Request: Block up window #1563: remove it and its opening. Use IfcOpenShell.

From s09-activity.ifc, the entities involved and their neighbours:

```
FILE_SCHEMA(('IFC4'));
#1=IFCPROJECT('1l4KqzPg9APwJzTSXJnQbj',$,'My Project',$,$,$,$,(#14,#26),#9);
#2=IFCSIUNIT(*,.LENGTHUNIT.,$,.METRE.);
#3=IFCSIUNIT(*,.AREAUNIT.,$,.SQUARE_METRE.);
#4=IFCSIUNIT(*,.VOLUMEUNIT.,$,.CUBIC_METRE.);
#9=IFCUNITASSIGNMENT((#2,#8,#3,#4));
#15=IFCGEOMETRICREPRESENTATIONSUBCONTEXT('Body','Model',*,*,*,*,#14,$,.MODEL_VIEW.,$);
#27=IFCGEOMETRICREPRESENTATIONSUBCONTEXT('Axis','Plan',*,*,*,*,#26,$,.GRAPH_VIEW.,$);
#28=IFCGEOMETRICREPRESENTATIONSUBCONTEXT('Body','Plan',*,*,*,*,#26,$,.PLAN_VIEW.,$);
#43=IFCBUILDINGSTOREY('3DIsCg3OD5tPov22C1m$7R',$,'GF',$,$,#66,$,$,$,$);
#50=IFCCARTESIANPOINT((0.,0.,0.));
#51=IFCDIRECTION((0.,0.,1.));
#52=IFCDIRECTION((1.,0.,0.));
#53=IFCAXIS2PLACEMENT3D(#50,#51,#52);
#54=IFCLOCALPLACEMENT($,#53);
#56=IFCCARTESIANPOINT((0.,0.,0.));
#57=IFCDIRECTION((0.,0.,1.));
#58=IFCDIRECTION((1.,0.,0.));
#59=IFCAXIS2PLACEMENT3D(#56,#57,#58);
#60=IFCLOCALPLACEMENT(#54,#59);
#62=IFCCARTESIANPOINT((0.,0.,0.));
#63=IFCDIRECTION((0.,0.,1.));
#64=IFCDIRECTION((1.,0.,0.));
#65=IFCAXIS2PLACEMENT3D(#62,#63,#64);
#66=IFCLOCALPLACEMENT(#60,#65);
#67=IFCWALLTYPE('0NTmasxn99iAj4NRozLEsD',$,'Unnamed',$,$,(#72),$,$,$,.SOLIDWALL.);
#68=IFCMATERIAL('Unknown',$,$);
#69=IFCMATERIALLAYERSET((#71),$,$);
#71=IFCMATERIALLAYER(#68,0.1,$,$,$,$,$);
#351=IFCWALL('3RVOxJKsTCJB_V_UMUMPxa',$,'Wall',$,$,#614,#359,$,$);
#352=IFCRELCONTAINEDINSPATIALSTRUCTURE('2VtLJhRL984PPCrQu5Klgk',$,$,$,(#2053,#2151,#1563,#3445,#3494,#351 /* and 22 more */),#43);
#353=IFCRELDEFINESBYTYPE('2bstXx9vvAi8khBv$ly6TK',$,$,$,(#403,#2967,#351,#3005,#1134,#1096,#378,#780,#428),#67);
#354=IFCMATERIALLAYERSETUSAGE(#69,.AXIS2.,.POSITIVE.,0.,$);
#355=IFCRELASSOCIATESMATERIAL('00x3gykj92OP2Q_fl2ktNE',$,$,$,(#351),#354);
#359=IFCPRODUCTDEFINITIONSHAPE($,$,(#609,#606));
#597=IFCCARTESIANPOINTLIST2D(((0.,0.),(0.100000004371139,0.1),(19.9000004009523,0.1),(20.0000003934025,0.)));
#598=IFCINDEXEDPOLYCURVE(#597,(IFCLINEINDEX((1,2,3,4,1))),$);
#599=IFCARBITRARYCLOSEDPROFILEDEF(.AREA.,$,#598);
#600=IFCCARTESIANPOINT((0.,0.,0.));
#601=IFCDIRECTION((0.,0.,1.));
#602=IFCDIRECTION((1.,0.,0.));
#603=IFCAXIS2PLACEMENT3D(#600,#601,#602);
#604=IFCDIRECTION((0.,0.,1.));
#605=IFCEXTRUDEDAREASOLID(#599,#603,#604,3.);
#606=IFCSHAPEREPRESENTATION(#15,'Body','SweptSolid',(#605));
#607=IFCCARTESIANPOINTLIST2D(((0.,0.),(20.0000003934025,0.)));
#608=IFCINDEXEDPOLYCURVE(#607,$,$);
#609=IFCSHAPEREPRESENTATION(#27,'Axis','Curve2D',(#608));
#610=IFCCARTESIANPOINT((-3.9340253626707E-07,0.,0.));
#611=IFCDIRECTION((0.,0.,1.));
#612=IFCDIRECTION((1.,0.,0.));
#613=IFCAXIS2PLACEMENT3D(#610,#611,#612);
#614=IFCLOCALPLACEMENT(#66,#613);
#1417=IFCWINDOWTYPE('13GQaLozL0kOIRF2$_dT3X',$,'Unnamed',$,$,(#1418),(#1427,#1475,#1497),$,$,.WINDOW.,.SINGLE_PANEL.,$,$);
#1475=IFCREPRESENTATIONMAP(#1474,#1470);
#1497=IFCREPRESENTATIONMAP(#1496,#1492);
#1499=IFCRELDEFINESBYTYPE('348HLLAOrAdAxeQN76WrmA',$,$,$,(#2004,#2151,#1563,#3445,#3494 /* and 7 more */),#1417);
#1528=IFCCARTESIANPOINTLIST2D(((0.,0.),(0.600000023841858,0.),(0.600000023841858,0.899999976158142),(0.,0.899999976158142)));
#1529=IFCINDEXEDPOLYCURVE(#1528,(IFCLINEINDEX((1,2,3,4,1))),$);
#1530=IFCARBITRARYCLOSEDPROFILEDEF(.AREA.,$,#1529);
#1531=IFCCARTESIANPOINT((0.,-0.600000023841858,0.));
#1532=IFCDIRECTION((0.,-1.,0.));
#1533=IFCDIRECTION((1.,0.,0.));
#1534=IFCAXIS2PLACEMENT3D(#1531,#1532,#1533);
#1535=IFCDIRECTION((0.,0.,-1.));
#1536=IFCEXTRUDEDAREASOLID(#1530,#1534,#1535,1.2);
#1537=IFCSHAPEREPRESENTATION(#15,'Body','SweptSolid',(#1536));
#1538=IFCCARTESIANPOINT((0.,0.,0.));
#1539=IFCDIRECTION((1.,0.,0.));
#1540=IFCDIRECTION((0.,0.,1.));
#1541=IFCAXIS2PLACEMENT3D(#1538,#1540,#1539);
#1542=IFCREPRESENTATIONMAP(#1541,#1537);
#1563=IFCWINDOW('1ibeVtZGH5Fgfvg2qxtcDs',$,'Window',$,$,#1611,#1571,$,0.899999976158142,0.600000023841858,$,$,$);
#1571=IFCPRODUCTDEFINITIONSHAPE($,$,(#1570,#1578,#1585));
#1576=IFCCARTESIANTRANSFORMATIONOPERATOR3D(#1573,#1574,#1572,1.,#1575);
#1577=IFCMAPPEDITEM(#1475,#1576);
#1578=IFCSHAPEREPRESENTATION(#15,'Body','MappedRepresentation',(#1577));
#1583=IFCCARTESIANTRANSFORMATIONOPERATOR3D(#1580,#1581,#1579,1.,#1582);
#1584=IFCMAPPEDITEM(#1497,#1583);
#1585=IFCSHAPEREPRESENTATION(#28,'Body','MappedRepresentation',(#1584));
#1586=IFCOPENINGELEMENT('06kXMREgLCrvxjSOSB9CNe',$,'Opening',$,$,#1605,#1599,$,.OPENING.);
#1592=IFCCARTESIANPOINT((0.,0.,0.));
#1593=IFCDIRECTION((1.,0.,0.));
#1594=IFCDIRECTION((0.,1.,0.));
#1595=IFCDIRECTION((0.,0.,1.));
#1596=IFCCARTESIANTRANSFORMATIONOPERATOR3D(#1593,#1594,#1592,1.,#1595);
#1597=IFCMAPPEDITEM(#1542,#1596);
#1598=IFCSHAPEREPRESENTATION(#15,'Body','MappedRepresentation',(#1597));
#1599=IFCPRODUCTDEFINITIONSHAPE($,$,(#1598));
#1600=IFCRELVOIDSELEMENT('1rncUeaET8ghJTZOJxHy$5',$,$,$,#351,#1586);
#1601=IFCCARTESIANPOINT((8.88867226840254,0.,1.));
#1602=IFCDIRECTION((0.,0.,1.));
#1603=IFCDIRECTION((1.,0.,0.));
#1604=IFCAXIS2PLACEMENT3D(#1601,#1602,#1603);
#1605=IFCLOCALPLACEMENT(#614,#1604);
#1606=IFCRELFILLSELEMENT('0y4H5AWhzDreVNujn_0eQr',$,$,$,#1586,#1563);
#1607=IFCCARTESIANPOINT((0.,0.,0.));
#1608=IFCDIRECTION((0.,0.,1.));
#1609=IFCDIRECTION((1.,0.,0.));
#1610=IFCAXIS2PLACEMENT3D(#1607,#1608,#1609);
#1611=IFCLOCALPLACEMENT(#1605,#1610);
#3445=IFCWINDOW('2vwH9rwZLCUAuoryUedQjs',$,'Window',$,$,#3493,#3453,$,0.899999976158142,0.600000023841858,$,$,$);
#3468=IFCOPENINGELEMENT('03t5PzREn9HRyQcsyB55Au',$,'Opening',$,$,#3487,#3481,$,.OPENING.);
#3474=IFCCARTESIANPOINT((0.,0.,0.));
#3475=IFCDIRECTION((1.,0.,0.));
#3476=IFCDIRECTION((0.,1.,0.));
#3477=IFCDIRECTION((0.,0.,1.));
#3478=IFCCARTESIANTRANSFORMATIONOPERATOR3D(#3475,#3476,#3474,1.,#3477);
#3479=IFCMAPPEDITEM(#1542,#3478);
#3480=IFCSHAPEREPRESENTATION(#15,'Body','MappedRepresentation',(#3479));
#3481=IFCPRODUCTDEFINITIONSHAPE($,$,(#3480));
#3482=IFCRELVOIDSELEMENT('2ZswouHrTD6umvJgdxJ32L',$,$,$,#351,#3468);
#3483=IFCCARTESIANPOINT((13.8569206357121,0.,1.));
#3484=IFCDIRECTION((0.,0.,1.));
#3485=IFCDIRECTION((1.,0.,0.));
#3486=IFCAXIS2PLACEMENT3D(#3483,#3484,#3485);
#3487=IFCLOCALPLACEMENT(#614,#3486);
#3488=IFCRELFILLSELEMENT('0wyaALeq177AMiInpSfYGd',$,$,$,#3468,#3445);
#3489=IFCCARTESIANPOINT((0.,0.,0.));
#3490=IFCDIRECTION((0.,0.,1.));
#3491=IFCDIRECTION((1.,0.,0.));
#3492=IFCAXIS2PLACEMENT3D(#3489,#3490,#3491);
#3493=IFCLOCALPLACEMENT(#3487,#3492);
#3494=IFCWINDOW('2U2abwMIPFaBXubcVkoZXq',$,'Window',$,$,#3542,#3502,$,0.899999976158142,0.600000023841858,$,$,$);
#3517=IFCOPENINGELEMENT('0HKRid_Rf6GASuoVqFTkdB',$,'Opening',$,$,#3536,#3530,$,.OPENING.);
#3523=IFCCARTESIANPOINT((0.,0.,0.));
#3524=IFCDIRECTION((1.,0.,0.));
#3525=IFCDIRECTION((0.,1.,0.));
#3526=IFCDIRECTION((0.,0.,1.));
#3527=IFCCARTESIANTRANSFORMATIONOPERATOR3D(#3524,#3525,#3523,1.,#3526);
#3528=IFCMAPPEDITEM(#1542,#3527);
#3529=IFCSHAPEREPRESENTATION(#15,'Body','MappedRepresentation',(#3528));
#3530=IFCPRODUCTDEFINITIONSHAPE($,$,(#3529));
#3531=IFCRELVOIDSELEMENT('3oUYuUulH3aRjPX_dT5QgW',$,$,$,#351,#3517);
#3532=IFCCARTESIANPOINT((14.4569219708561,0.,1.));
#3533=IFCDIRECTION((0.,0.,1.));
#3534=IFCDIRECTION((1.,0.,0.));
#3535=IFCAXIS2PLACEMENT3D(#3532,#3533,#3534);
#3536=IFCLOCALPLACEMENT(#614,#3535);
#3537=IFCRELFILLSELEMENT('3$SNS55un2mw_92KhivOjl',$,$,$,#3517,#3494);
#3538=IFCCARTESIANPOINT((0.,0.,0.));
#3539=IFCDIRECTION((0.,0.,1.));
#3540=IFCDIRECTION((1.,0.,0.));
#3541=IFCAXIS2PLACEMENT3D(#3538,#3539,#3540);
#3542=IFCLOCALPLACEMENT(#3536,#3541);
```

```python
import ifcopenshell
import ifcopenshell.api.feature
import ifcopenshell.api.root
import ifcopenshell.geom
import ifcopenshell.util.shape

model = ifcopenshell.open("s09-activity.ifc")
settings = ifcopenshell.geom.settings()


def volume(element):
    """Net volume in cubic metres, openings subtracted."""
    shape = ifcopenshell.geom.create_shape(settings, element)
    return ifcopenshell.util.shape.get_volume(shape.geometry)


window = model.by_guid("1ibeVtZGH5Fgfvg2qxtcDs")
opening = window.FillsVoids[0].RelatingOpeningElement
wall = opening.VoidsElements[0].RelatingBuildingElement
before = volume(wall)

ifcopenshell.api.root.remove_product(model, product=window)
ifcopenshell.api.feature.remove_feature(model, feature=opening)

after = volume(wall)

print(f"wall volume {before:.3f} -> {after:.3f} m3")

model.write("s09-activity-out.ifc")
```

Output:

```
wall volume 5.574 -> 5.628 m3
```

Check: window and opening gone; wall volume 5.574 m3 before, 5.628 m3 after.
